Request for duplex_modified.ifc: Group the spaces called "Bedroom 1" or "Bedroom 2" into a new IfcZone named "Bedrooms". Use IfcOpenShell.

First a look at what the model holds.

```python
import ifcopenshell

model = ifcopenshell.open("duplex_modified.ifc")
print(model.schema)
seen = {}
for space in model.by_type("IfcSpace"):
    seen[space.LongName] = seen.get(space.LongName, 0) + 1
for name, count in sorted(seen.items(), key=str):
    print(count, "x", name)
print("zones:", [z.Name for z in model.by_type("IfcZone")][:20])
```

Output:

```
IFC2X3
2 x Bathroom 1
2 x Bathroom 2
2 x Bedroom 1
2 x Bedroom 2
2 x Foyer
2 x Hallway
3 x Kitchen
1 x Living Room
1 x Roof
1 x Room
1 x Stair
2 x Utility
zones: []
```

```python
import ifcopenshell
import ifcopenshell.api.group
import ifcopenshell.api.root

model = ifcopenshell.open("duplex_modified.ifc")

names = {"Bedroom 1", "Bedroom 2"}
spaces = [s for s in model.by_type("IfcSpace") if s.LongName in names]

zone = ifcopenshell.api.root.create_entity(model, ifc_class="IfcZone", name="Bedrooms")
ifcopenshell.api.group.assign_group(model, products=spaces, group=zone)
print(len(spaces), "spaces in", zone.Name)

model.write("duplex_modified_rev.ifc")
```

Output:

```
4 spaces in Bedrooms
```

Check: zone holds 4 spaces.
